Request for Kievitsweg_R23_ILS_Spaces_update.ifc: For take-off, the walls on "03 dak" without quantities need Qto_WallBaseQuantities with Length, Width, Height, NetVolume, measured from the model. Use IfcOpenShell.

First a look at what the model holds.

```python
import ifcopenshell
import ifcopenshell.util.element
import ifcopenshell.util.unit

model = ifcopenshell.open("Kievitsweg_R23_ILS_Spaces_update.ifc")
print(model.schema)
for unit_type in ("LENGTHUNIT", "AREAUNIT", "VOLUMEUNIT"):
    print(unit_type, ifcopenshell.util.unit.calculate_unit_scale(model, unit_type))
storey = next(s for s in model.by_type("IfcBuildingStorey") if s.Name == "03 dak")
walls = [e for e in ifcopenshell.util.element.get_decomposition(storey) if e.is_a("IfcWall")]
for e in sorted(walls, key=lambda e: e.id()):
    print(e.id(), e.is_a(), e.Name, list(ifcopenshell.util.element.get_psets(e, qtos_only=True)), sep=" | ")
```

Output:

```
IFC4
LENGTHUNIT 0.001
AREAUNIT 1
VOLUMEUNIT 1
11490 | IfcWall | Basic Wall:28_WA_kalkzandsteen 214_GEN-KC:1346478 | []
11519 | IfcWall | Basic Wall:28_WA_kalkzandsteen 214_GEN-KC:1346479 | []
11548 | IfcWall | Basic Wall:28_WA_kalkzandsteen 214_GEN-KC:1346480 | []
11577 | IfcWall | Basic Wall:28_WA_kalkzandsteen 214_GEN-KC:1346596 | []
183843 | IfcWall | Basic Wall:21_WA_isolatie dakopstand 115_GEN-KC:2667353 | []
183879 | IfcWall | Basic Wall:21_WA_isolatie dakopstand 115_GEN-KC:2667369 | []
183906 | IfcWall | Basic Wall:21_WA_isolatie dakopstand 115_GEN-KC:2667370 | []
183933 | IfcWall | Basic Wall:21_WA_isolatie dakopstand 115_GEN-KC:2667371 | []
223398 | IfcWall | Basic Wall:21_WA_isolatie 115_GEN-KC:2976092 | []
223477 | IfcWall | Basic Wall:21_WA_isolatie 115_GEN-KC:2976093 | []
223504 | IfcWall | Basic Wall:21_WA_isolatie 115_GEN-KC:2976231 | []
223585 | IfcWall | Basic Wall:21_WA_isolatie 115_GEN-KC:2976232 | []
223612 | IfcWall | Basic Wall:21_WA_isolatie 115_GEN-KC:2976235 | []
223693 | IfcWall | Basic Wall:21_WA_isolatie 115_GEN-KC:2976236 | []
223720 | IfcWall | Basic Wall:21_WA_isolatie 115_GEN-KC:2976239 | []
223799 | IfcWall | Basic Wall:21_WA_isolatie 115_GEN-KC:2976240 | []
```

```python
import ifcopenshell
import ifcopenshell.api.pset
import ifcopenshell.geom
import ifcopenshell.util.element
import ifcopenshell.util.shape
import ifcopenshell.util.unit

model = ifcopenshell.open("Kievitsweg_R23_ILS_Spaces_update.ifc")
unit_scale = ifcopenshell.util.unit.calculate_unit_scale(model)
volume_scale = ifcopenshell.util.unit.calculate_unit_scale(model, "VOLUMEUNIT")
settings = ifcopenshell.geom.settings()

storey = next(s for s in model.by_type("IfcBuildingStorey") if s.Name == "03 dak")
walls = [e for e in ifcopenshell.util.element.get_decomposition(storey) if e.is_a("IfcWall")]

for e in sorted(walls, key=lambda e: e.id()):
    if ifcopenshell.util.element.get_psets(e, qtos_only=True, should_inherit=False):
        continue
    # Geometry comes back in metres, in the element's own axes.
    shape = ifcopenshell.geom.create_shape(settings, e)
    values = {
        "Length": ifcopenshell.util.shape.get_x(shape.geometry) / unit_scale,
        "Width": ifcopenshell.util.shape.get_y(shape.geometry) / unit_scale,
        "Height": ifcopenshell.util.shape.get_z(shape.geometry) / unit_scale,
        "NetVolume": ifcopenshell.util.shape.get_volume(shape.geometry) / volume_scale,
    }
    qto = ifcopenshell.api.pset.add_qto(model, product=e, name="Qto_WallBaseQuantities")
    ifcopenshell.api.pset.edit_qto(model, qto=qto, properties=values)
    print(e.id(), {k: round(v, 3) for k, v in values.items()})

model.write("Kievitsweg_R23_ILS_Spaces_update_updated.ifc")
```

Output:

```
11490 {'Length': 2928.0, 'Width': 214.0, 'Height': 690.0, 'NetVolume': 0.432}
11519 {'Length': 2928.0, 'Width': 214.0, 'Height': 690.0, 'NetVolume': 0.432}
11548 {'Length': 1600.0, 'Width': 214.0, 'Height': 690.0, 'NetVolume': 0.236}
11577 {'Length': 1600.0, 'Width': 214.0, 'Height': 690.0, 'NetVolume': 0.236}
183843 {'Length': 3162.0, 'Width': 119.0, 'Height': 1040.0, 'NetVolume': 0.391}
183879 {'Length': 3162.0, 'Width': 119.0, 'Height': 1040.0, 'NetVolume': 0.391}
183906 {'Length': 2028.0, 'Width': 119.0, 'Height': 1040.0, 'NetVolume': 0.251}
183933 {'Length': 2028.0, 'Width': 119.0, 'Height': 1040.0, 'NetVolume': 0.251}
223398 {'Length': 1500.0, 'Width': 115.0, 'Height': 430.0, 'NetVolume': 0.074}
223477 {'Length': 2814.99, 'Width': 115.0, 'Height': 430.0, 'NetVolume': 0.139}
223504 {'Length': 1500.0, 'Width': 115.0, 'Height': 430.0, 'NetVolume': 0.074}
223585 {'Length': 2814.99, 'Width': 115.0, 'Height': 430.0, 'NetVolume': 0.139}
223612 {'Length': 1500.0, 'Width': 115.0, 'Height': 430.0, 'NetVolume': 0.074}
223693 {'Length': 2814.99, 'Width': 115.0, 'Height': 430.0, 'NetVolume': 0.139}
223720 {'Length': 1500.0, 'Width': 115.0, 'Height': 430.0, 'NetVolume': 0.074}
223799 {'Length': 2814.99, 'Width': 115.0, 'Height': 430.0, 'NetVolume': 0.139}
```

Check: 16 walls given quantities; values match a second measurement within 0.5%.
